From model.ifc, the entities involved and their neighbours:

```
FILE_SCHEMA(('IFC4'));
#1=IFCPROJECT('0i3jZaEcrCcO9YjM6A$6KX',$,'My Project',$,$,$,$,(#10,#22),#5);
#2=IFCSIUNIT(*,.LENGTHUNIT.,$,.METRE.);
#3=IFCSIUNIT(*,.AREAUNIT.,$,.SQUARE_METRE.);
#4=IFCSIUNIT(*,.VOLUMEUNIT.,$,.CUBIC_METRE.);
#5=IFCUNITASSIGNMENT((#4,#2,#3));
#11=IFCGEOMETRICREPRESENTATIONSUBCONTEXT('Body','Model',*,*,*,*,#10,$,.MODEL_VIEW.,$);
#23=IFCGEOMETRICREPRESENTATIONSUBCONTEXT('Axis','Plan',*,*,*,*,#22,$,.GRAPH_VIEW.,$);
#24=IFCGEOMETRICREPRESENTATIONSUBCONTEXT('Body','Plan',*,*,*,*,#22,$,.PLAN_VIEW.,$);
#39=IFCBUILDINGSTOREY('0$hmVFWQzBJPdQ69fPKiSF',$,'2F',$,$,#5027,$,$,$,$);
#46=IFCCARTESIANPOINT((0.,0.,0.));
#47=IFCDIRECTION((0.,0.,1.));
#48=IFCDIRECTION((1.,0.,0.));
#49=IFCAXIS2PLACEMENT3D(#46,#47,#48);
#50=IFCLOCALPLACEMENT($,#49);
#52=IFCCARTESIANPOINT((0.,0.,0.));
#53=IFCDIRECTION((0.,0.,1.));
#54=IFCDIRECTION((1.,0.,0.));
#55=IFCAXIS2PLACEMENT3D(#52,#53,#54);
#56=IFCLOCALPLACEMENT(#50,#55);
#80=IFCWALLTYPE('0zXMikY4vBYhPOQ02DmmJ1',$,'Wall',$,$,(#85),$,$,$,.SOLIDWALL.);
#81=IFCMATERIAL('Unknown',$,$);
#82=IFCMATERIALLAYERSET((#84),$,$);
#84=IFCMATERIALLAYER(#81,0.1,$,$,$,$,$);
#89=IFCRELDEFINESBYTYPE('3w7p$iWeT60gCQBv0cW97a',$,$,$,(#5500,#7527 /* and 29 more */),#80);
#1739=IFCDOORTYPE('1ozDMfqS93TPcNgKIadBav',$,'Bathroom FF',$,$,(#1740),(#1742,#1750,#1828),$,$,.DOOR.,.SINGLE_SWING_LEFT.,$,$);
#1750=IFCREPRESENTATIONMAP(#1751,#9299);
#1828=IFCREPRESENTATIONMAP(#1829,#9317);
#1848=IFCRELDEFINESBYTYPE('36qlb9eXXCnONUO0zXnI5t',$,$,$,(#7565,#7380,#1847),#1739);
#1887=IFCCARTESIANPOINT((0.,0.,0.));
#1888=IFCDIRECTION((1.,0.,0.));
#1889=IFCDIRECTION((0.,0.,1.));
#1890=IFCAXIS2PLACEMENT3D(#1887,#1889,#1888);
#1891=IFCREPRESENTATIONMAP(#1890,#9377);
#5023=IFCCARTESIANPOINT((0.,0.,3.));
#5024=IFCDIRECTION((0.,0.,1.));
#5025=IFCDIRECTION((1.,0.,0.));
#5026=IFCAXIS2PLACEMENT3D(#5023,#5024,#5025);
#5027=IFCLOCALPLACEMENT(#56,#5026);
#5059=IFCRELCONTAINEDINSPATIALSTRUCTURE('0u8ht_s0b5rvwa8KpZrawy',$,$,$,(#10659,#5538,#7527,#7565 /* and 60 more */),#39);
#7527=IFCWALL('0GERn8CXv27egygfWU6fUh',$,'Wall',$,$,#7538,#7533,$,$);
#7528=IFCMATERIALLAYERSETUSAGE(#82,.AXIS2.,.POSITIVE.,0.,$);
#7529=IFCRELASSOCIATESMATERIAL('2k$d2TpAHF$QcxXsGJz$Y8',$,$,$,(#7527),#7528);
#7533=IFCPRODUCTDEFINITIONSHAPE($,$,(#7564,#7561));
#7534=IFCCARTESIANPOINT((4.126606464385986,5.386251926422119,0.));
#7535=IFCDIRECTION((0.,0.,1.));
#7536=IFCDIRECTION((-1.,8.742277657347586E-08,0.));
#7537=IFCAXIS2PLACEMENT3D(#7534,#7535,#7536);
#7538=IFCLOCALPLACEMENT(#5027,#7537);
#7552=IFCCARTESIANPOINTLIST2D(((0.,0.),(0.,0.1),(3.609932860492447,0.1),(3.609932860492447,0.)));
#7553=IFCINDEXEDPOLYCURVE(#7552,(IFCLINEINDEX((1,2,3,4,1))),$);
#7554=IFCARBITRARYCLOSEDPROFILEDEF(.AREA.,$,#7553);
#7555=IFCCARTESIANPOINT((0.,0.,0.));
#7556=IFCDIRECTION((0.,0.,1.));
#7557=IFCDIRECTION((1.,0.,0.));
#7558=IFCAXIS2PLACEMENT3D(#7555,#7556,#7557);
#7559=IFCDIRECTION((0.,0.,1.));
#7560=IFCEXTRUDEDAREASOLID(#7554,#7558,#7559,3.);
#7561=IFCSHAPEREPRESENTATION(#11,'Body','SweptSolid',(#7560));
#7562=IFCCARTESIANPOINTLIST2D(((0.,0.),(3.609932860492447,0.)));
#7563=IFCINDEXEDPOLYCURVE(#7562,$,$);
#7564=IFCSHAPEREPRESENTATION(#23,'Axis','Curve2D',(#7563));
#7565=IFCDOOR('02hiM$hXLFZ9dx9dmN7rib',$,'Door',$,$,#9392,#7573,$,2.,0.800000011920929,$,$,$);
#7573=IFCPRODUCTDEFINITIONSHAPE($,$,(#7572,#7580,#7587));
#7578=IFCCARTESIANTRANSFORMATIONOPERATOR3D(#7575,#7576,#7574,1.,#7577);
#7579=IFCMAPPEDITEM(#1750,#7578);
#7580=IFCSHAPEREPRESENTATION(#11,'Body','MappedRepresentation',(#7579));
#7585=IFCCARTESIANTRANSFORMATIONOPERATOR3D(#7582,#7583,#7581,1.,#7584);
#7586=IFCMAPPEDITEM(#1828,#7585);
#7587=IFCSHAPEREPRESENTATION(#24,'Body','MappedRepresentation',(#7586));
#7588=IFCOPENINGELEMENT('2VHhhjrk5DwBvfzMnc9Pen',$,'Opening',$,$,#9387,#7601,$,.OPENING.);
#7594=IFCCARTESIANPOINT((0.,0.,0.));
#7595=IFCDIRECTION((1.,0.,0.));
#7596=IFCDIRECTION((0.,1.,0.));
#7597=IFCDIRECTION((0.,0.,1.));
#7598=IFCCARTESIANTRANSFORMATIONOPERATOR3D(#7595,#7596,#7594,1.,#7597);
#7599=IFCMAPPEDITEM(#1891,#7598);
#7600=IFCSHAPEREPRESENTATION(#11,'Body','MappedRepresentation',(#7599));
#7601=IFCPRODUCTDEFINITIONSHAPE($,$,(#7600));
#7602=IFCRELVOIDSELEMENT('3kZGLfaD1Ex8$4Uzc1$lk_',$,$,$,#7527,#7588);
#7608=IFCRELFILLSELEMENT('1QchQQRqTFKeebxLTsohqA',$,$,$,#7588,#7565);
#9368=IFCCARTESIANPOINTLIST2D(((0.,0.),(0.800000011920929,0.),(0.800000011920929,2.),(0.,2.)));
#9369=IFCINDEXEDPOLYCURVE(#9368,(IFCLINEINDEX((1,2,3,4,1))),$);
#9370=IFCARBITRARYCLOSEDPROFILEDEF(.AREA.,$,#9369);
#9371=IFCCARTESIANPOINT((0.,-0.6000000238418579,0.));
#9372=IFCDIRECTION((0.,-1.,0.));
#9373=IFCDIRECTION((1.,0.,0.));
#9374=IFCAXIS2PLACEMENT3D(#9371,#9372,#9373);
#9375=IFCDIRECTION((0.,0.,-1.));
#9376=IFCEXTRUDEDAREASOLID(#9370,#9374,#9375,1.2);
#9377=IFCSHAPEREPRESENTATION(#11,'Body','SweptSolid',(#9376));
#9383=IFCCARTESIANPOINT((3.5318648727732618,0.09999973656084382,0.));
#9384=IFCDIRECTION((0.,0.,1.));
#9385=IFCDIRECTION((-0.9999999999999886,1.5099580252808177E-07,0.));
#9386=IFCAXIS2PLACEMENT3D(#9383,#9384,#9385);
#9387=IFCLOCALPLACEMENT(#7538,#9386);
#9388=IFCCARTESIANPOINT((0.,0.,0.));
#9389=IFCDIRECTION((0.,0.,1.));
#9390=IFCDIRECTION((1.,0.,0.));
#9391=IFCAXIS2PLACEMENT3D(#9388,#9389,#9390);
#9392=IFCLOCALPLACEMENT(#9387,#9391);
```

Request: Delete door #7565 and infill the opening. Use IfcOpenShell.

```python
import ifcopenshell
import ifcopenshell.api.feature
import ifcopenshell.api.root
import ifcopenshell.geom
import ifcopenshell.util.shape

model = ifcopenshell.open("model.ifc")
settings = ifcopenshell.geom.settings()


def volume(element):
    """Net volume in cubic metres, openings subtracted."""
    shape = ifcopenshell.geom.create_shape(settings, element)
    return ifcopenshell.util.shape.get_volume(shape.geometry)


door = model.by_guid("02hiM$hXLFZ9dx9dmN7rib")
opening = door.FillsVoids[0].RelatingOpeningElement
wall = opening.VoidsElements[0].RelatingBuildingElement
before = volume(wall)

ifcopenshell.api.root.remove_product(model, product=door)
ifcopenshell.api.feature.remove_feature(model, feature=opening)

after = volume(wall)

print(f"wall volume {before:.3f} -> {after:.3f} m3")

model.write("model-out.ifc")
```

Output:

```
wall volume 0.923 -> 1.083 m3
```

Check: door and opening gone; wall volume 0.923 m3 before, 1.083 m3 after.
